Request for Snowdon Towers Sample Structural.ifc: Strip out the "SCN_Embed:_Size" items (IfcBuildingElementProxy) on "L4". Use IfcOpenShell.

First a look at what the model holds.

```python
import ifcopenshell
import ifcopenshell.util.element

model = ifcopenshell.open("Snowdon Towers Sample Structural.ifc")
print(model.schema)
storey = next(s for s in model.by_type("IfcBuildingStorey") if s.Name == "L4")
proxies = [e for e in ifcopenshell.util.element.get_decomposition(storey) if e.is_a("IfcBuildingElementProxy")]
seen = {}
for e in proxies:
    element_type = ifcopenshell.util.element.get_type(e)
    name = element_type.Name if element_type not in (None, e) else None
    seen[name] = seen.get(name, 0) + 1
for name, count in sorted(seen.items(), key=str):
    print(count, "x", name)
```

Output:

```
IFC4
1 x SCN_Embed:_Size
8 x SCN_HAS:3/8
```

```python
import ifcopenshell
import ifcopenshell.api.root
import ifcopenshell.util.element

model = ifcopenshell.open("Snowdon Towers Sample Structural.ifc")

storey = next(s for s in model.by_type("IfcBuildingStorey") if s.Name == "L4")
proxies = [e for e in ifcopenshell.util.element.get_decomposition(storey) if e.is_a("IfcBuildingElementProxy")]
targets = [e for e in proxies if (t := ifcopenshell.util.element.get_type(e)) not in (None, e) and t.Name == "SCN_Embed:_Size"]

for e in targets:
    ifcopenshell.api.root.remove_product(model, product=e)
print(len(targets), "removed")

model.write("Snowdon Towers Sample Structural-out.ifc")
```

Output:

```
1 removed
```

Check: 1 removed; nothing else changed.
